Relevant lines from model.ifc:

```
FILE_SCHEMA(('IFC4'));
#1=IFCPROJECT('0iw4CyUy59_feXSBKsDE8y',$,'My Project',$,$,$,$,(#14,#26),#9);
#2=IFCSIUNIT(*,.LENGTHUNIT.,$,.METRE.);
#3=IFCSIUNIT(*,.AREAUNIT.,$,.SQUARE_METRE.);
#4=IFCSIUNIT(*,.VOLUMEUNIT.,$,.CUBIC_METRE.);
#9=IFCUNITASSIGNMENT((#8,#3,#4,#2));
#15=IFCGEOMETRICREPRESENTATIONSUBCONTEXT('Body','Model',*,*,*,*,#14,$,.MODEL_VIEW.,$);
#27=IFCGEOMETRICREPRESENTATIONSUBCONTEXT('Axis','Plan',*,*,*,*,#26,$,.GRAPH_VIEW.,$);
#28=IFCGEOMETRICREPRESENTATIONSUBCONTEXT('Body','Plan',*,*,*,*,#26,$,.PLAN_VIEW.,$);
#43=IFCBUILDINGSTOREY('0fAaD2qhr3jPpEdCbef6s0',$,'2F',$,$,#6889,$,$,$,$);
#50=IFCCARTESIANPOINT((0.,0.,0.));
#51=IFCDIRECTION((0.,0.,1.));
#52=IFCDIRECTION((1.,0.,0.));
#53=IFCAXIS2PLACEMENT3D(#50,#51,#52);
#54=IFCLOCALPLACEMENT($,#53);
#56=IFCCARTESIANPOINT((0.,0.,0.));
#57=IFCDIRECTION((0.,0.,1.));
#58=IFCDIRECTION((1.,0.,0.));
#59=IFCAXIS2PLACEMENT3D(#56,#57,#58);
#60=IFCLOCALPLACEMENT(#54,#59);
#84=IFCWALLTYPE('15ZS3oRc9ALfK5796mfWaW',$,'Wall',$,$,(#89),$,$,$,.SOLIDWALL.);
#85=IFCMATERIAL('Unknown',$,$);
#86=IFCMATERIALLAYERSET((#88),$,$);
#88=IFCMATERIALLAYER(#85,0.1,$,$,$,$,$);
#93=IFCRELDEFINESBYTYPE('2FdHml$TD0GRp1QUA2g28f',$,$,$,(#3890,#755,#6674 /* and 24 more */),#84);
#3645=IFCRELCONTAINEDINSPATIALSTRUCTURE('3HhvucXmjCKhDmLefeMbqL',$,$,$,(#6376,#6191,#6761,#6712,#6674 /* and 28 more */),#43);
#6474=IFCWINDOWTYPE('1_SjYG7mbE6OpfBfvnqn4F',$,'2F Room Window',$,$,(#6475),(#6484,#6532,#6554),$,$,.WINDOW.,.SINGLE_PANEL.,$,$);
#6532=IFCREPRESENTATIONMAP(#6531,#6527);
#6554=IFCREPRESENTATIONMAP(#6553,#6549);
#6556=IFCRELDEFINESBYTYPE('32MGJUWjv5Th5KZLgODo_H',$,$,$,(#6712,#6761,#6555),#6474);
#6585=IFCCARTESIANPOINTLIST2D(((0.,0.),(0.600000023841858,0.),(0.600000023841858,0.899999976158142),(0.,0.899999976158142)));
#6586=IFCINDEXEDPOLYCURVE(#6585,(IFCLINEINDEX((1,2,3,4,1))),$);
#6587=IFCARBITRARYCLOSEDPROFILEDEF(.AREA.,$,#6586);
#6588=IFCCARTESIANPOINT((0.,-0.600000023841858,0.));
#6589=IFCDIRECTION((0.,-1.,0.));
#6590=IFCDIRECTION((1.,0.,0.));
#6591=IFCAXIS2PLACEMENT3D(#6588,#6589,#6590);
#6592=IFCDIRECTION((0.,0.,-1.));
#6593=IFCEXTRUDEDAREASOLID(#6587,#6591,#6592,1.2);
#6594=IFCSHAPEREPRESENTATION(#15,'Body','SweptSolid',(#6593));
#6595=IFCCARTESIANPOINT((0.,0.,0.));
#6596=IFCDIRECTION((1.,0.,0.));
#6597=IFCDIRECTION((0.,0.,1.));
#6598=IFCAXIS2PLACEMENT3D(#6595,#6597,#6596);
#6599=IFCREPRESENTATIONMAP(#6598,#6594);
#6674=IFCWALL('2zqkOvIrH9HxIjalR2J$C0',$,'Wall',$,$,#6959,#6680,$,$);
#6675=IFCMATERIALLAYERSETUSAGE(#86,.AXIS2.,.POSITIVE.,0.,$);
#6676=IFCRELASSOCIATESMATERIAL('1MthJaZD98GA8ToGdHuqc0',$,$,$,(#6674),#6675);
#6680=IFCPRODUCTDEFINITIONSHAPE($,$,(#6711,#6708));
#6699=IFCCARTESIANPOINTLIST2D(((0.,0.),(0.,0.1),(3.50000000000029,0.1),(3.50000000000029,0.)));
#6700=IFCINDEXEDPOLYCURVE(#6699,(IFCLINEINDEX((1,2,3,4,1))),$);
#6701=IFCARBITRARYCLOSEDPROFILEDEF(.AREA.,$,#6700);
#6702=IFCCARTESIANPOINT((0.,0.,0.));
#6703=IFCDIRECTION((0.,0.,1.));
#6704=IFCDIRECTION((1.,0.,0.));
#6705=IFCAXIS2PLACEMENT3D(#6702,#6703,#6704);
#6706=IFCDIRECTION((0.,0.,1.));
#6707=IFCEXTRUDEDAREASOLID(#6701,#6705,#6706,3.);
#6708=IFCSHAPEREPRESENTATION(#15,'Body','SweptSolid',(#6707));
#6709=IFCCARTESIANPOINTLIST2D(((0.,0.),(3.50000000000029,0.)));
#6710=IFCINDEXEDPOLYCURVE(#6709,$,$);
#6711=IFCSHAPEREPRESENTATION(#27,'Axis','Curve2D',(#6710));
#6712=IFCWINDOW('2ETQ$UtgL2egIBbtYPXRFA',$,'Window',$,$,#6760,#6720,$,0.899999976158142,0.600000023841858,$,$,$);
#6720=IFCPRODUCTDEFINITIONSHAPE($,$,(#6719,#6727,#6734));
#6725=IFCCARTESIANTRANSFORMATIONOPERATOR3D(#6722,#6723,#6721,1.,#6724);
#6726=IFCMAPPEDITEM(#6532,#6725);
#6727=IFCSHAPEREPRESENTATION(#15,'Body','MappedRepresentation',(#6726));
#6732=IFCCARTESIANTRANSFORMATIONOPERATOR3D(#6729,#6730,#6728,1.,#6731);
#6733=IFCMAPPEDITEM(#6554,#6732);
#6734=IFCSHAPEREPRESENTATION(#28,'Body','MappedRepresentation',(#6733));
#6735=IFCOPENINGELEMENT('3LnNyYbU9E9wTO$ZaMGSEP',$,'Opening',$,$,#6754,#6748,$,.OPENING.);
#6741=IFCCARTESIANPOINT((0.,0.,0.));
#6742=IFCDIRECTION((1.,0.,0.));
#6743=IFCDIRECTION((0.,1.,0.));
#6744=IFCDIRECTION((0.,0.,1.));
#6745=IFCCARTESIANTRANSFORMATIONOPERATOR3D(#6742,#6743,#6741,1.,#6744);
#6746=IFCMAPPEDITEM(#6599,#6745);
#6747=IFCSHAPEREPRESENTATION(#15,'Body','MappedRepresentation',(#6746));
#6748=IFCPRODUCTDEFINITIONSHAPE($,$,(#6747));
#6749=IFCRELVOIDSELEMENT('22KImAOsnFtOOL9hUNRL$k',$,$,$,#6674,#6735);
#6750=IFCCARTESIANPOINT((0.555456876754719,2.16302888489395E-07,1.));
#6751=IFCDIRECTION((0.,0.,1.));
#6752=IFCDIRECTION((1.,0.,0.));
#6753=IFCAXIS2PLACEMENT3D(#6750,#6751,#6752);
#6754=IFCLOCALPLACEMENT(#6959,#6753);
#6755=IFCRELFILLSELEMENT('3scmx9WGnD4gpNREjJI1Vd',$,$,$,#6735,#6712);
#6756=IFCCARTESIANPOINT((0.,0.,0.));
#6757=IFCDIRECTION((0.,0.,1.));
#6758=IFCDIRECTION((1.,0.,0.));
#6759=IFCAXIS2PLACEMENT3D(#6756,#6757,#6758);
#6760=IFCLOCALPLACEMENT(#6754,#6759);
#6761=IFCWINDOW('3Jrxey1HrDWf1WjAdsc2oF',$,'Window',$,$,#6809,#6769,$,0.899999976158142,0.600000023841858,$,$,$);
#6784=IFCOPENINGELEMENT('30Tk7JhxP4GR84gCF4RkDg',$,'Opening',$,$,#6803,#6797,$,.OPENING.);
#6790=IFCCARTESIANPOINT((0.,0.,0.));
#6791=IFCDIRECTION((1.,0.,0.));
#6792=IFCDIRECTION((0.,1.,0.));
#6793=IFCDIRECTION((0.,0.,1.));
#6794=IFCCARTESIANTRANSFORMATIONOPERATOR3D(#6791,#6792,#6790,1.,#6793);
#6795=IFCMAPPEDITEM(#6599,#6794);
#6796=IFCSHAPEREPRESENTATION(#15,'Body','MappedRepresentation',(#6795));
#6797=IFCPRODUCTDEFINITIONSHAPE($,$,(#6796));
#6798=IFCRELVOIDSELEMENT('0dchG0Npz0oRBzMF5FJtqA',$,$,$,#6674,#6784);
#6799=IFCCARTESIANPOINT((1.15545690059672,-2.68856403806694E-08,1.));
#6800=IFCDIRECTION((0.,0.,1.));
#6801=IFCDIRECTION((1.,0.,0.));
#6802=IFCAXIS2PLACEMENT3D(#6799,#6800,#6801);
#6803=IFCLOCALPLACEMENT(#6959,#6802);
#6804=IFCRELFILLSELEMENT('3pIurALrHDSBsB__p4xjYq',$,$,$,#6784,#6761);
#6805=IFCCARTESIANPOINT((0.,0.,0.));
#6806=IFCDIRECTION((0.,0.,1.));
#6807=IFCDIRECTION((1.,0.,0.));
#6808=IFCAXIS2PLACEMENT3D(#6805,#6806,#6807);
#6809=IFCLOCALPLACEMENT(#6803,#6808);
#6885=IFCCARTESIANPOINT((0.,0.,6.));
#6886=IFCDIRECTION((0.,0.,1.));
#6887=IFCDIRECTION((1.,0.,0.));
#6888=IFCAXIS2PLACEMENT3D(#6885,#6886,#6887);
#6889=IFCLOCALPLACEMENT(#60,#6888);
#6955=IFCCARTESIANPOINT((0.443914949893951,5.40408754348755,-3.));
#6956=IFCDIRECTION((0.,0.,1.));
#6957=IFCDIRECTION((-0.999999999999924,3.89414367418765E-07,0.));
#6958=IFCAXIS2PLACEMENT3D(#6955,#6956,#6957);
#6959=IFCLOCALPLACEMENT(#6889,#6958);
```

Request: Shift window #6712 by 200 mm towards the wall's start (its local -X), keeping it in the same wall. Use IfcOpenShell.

```python
import ifcopenshell
import ifcopenshell.api.geometry
import ifcopenshell.util.placement

model = ifcopenshell.open("model.ifc")

window = model.by_guid("2ETQ$UtgL2egIBbtYPXRFA")
opening = window.FillsVoids[0].RelatingOpeningElement
wall = opening.VoidsElements[0].RelatingBuildingElement

wall_matrix = ifcopenshell.util.placement.get_local_placement(wall.ObjectPlacement)
shift = wall_matrix[:3, 0] * -0.2
before = ifcopenshell.util.placement.get_local_placement(window.ObjectPlacement)[:3, 3].copy()

# The window is placed relative to its opening, so it follows when the opening moves.
matrix = ifcopenshell.util.placement.get_local_placement(opening.ObjectPlacement)
matrix[:3, 3] += shift
ifcopenshell.api.geometry.edit_object_placement(
    model, product=opening, matrix=matrix, is_si=False, should_transform_children=True
)

after = ifcopenshell.util.placement.get_local_placement(window.ObjectPlacement)[:3, 3]
print("window moved by", (after - before).round(3) + 0.0)

model.write("model_updated.ifc")
```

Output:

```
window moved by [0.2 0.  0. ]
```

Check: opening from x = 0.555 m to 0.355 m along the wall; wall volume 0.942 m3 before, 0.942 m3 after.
